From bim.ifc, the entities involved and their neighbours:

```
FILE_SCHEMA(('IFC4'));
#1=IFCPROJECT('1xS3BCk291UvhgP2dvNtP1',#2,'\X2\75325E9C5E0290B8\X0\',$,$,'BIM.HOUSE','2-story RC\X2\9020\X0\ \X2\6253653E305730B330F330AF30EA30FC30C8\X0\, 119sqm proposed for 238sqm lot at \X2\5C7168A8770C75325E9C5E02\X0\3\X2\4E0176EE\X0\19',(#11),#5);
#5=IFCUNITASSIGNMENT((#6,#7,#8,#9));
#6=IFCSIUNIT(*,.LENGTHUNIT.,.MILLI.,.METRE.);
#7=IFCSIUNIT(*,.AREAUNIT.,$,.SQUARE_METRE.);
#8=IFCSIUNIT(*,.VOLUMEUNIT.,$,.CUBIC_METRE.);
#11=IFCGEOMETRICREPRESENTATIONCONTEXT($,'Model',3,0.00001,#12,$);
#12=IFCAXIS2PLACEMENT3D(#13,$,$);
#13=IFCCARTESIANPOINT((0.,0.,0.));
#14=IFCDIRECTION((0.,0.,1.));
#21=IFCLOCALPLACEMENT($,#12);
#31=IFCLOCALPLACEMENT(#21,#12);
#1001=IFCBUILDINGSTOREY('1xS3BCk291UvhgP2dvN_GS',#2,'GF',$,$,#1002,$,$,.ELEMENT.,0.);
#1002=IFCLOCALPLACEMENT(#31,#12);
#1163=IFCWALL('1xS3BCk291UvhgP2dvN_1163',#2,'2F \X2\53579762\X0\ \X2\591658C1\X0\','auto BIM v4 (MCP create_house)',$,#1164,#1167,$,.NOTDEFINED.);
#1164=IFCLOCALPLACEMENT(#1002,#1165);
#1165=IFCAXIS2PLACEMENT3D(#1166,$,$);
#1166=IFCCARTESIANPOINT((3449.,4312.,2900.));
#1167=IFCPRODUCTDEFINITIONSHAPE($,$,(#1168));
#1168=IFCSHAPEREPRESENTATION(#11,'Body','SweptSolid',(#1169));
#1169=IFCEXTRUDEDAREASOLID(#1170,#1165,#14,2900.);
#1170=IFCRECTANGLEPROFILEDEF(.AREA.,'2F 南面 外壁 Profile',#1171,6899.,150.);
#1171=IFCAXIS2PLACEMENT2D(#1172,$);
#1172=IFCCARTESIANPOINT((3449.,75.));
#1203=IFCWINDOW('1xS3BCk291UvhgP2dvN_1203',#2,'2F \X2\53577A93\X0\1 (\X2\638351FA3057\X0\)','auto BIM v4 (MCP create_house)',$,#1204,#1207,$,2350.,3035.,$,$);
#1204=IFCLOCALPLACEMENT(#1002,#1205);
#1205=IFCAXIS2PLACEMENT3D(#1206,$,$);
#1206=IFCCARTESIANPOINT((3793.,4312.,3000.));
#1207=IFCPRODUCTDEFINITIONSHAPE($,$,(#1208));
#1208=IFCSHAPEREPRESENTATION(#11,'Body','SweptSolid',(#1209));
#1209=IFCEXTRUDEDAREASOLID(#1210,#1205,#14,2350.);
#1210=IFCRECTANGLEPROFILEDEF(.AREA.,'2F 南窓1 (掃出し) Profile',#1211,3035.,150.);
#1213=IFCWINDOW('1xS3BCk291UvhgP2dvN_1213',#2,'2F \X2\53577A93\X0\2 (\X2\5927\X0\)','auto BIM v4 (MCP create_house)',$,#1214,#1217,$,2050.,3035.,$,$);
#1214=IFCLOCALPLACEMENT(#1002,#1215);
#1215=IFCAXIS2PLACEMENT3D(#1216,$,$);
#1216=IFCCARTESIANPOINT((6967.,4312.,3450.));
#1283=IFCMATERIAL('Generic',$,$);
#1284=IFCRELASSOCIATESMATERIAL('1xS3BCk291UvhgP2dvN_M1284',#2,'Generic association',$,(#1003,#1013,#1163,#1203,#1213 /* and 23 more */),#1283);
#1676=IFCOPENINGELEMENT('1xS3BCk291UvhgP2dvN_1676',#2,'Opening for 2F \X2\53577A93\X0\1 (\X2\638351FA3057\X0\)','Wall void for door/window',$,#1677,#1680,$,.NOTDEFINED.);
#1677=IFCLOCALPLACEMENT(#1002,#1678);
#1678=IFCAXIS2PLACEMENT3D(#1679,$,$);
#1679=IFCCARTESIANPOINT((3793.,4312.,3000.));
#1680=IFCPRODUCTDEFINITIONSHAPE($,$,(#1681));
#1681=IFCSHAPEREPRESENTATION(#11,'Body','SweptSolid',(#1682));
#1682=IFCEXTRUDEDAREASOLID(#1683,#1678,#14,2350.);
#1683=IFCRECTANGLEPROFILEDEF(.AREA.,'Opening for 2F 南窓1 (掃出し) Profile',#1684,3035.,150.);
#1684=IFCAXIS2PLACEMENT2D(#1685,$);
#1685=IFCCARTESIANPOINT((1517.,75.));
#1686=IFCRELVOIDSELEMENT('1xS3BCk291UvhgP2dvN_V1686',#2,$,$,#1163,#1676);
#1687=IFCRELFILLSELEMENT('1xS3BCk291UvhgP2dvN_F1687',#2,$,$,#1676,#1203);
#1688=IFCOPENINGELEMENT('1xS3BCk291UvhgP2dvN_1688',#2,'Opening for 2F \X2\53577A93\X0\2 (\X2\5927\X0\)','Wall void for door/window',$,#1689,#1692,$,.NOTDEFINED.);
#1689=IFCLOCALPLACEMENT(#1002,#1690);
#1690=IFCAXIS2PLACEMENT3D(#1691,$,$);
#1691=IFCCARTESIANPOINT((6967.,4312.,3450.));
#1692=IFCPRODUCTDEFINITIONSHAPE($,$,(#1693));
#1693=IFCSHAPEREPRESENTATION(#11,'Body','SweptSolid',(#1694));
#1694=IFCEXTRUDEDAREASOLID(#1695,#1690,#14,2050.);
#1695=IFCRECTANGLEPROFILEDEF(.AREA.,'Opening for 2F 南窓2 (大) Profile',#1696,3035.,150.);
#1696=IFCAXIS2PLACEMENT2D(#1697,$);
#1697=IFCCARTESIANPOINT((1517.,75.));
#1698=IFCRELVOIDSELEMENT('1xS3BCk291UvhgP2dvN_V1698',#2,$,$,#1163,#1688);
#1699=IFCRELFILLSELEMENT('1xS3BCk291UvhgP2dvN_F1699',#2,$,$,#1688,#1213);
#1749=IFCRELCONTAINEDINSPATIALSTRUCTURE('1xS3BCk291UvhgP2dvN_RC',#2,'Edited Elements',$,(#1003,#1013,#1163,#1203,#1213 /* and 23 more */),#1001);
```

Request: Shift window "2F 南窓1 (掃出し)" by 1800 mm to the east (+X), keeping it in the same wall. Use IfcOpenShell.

```python
import ifcopenshell
import ifcopenshell.api.geometry
import ifcopenshell.util.placement

model = ifcopenshell.open("bim.ifc")

window = model.by_guid("1xS3BCk291UvhgP2dvN_1203")
opening = window.FillsVoids[0].RelatingOpeningElement
wall = opening.VoidsElements[0].RelatingBuildingElement

wall_matrix = ifcopenshell.util.placement.get_local_placement(wall.ObjectPlacement)
shift = wall_matrix[:3, 0] * 1800.0
before = ifcopenshell.util.placement.get_local_placement(window.ObjectPlacement)[:3, 3].copy()

# The window is not placed relative to its opening, so move both.
for product in (opening, window):
    matrix = ifcopenshell.util.placement.get_local_placement(product.ObjectPlacement)
    matrix[:3, 3] += shift
    ifcopenshell.api.geometry.edit_object_placement(model, product=product, matrix=matrix, is_si=False)

after = ifcopenshell.util.placement.get_local_placement(window.ObjectPlacement)[:3, 3]
print("window moved by", (after - before).round(3) + 0.0)

model.write("bim_edited.ifc")
```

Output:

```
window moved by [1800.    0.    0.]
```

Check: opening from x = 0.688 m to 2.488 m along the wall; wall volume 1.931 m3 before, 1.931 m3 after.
